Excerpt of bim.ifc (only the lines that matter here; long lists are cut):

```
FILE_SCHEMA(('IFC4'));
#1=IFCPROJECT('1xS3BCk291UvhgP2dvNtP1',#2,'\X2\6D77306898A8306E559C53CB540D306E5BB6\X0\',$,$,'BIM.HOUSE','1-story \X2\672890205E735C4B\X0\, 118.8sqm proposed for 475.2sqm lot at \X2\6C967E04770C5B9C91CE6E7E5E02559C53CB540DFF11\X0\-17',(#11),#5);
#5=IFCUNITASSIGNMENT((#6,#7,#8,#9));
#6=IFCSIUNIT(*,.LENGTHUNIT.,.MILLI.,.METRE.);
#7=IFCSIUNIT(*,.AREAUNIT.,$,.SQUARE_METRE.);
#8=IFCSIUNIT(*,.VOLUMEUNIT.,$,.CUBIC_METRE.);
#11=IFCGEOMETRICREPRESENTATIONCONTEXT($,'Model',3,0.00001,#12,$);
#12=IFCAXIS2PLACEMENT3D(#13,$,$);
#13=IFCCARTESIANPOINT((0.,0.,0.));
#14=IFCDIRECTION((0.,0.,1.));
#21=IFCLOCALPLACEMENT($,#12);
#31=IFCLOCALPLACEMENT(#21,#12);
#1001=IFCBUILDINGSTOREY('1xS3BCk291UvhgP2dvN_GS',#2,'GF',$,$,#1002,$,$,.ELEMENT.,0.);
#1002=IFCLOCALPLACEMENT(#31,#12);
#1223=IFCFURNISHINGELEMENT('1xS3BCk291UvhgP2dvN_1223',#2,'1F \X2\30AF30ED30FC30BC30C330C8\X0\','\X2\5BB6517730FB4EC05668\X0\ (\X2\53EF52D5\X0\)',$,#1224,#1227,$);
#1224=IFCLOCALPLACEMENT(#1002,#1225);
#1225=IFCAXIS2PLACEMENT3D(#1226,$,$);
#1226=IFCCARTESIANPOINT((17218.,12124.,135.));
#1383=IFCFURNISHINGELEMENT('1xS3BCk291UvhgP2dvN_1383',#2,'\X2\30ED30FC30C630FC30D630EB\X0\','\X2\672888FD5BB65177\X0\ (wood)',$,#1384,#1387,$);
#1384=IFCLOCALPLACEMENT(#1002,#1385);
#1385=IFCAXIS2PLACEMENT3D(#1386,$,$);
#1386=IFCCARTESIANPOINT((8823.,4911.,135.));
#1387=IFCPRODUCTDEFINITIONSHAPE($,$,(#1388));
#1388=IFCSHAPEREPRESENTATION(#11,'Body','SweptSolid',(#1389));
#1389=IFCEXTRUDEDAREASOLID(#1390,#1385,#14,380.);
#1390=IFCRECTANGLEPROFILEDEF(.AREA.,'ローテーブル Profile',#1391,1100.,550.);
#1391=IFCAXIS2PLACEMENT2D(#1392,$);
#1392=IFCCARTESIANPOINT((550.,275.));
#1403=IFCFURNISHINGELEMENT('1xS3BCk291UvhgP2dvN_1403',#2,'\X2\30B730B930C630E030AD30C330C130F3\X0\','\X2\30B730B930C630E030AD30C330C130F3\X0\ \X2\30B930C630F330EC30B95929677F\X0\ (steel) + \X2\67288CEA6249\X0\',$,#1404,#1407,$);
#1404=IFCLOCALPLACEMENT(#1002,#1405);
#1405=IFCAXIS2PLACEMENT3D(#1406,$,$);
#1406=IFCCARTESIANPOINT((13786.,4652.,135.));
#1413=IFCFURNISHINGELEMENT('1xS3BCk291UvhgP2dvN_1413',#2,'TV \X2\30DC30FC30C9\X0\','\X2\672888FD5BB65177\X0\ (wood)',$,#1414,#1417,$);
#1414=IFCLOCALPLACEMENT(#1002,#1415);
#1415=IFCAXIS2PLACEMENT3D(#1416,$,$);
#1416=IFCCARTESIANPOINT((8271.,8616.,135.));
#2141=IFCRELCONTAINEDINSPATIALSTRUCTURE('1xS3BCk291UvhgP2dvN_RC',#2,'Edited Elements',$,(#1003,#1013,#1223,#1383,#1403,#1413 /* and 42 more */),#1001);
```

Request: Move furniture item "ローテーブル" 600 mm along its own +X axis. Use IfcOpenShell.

```python
import ifcopenshell
import ifcopenshell.api.geometry
import ifcopenshell.util.placement

model = ifcopenshell.open("bim.ifc")

item = model.by_guid("1xS3BCk291UvhgP2dvN_1383")
matrix = ifcopenshell.util.placement.get_local_placement(item.ObjectPlacement)
matrix[:3, 3] += matrix[:3, 0] * 600.0
ifcopenshell.api.geometry.edit_object_placement(model, product=item, matrix=matrix, is_si=False)

print(ifcopenshell.util.placement.get_local_placement(item.ObjectPlacement).round(3) + 0.0)

model.write("bim-out.ifc")
```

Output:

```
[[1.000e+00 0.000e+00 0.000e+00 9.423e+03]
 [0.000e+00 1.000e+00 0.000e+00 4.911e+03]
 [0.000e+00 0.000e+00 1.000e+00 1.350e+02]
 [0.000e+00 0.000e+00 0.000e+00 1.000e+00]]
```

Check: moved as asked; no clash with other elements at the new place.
